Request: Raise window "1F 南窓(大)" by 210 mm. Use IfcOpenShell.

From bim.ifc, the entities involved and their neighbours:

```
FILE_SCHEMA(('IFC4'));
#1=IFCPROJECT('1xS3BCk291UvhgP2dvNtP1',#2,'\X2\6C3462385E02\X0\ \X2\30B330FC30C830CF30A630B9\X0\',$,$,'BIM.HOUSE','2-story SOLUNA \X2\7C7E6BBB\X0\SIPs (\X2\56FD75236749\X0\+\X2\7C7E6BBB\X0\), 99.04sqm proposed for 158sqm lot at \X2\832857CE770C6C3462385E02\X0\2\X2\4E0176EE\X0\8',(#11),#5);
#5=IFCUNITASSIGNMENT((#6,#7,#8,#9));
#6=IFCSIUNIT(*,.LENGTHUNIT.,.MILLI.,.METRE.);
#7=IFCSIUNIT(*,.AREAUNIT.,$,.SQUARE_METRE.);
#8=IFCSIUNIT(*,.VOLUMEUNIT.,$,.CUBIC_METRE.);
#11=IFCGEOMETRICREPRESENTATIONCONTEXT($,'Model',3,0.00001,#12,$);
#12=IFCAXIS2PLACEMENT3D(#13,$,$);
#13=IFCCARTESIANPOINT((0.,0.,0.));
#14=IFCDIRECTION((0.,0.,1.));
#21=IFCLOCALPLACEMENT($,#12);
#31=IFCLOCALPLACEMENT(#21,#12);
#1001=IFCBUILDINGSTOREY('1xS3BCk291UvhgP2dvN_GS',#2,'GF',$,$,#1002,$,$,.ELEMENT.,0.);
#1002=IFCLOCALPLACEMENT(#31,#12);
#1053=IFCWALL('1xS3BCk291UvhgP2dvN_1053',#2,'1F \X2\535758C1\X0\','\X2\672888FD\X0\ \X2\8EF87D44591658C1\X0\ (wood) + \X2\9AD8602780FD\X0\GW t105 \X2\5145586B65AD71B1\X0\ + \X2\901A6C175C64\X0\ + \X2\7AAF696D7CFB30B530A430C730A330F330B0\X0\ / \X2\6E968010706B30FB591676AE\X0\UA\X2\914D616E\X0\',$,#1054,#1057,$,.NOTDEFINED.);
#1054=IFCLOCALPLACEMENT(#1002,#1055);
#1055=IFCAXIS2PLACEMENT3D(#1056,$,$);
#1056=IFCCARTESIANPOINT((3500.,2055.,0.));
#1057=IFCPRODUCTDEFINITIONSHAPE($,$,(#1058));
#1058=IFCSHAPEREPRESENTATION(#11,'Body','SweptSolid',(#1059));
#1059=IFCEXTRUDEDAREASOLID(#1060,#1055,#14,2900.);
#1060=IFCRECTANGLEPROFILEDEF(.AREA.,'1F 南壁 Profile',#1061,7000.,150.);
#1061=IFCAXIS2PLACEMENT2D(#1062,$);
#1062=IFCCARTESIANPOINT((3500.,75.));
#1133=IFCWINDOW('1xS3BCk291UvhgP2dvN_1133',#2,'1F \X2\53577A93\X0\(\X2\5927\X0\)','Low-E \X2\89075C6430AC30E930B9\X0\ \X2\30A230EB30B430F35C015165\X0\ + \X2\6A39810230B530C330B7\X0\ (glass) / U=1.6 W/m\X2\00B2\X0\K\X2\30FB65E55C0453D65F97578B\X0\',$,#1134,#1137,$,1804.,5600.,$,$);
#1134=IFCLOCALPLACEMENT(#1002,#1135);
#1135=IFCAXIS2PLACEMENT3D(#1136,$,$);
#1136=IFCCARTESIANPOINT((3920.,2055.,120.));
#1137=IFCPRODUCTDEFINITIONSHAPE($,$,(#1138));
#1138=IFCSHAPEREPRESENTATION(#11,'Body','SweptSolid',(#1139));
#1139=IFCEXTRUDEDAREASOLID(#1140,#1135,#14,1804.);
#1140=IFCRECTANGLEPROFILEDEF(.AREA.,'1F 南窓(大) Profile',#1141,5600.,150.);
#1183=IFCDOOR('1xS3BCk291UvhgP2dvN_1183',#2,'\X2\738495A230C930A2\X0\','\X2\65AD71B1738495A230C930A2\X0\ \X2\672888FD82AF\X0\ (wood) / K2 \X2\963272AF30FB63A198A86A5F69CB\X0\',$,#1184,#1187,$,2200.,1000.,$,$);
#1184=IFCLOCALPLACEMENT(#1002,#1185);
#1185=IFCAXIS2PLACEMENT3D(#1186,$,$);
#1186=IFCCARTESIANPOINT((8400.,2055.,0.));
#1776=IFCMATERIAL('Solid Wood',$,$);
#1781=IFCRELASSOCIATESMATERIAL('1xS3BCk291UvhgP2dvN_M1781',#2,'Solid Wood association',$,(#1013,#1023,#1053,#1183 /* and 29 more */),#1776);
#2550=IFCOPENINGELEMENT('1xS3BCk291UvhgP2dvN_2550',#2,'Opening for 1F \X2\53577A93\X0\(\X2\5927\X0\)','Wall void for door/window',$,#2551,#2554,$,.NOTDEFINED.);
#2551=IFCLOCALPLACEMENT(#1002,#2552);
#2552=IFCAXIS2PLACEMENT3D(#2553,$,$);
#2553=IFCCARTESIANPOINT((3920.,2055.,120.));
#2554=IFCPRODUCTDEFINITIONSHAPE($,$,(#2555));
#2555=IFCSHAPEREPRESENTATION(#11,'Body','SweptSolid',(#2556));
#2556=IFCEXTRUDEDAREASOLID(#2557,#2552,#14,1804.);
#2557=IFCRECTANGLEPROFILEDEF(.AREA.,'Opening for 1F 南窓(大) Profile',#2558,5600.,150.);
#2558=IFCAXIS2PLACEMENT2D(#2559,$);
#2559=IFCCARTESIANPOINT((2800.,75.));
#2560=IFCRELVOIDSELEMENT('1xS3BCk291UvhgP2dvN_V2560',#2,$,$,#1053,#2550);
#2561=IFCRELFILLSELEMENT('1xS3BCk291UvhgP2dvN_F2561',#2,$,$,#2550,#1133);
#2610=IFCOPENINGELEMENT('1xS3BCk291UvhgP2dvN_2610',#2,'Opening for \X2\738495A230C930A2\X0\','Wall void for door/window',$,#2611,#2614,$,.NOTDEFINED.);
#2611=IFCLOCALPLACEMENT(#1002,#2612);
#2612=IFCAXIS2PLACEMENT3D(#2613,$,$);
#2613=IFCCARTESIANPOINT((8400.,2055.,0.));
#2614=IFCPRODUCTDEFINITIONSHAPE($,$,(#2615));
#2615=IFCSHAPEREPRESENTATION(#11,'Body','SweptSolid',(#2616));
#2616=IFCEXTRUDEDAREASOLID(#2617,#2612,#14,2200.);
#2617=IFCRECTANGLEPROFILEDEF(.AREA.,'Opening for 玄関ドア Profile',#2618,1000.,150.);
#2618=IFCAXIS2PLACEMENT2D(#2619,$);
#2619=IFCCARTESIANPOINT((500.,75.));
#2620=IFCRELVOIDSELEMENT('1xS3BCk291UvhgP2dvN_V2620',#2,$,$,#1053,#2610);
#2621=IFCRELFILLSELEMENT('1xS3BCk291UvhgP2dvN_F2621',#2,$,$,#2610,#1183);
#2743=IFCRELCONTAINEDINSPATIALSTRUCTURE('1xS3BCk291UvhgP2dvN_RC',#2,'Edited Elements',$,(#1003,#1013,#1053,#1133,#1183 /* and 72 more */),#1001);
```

```python
import numpy as np
import ifcopenshell
import ifcopenshell.api.geometry
import ifcopenshell.util.placement
import ifcopenshell.util.unit

model = ifcopenshell.open("bim.ifc")
unit_scale = ifcopenshell.util.unit.calculate_unit_scale(model)

window = model.by_guid("1xS3BCk291UvhgP2dvN_1133")
opening = window.FillsVoids[0].RelatingOpeningElement
dz = 0.21 / unit_scale

shift = np.array([0.0, 0.0, dz])
# The window is not placed relative to its opening, so move both.
for product in (opening, window):
    matrix = ifcopenshell.util.placement.get_local_placement(product.ObjectPlacement)
    matrix[:3, 3] += shift
    ifcopenshell.api.geometry.edit_object_placement(model, product=product, matrix=matrix, is_si=False)

print(f"moved by {dz * unit_scale:+.3f} m")

model.write("bim-out.ifc")
```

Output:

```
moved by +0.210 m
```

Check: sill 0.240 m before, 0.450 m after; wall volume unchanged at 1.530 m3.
